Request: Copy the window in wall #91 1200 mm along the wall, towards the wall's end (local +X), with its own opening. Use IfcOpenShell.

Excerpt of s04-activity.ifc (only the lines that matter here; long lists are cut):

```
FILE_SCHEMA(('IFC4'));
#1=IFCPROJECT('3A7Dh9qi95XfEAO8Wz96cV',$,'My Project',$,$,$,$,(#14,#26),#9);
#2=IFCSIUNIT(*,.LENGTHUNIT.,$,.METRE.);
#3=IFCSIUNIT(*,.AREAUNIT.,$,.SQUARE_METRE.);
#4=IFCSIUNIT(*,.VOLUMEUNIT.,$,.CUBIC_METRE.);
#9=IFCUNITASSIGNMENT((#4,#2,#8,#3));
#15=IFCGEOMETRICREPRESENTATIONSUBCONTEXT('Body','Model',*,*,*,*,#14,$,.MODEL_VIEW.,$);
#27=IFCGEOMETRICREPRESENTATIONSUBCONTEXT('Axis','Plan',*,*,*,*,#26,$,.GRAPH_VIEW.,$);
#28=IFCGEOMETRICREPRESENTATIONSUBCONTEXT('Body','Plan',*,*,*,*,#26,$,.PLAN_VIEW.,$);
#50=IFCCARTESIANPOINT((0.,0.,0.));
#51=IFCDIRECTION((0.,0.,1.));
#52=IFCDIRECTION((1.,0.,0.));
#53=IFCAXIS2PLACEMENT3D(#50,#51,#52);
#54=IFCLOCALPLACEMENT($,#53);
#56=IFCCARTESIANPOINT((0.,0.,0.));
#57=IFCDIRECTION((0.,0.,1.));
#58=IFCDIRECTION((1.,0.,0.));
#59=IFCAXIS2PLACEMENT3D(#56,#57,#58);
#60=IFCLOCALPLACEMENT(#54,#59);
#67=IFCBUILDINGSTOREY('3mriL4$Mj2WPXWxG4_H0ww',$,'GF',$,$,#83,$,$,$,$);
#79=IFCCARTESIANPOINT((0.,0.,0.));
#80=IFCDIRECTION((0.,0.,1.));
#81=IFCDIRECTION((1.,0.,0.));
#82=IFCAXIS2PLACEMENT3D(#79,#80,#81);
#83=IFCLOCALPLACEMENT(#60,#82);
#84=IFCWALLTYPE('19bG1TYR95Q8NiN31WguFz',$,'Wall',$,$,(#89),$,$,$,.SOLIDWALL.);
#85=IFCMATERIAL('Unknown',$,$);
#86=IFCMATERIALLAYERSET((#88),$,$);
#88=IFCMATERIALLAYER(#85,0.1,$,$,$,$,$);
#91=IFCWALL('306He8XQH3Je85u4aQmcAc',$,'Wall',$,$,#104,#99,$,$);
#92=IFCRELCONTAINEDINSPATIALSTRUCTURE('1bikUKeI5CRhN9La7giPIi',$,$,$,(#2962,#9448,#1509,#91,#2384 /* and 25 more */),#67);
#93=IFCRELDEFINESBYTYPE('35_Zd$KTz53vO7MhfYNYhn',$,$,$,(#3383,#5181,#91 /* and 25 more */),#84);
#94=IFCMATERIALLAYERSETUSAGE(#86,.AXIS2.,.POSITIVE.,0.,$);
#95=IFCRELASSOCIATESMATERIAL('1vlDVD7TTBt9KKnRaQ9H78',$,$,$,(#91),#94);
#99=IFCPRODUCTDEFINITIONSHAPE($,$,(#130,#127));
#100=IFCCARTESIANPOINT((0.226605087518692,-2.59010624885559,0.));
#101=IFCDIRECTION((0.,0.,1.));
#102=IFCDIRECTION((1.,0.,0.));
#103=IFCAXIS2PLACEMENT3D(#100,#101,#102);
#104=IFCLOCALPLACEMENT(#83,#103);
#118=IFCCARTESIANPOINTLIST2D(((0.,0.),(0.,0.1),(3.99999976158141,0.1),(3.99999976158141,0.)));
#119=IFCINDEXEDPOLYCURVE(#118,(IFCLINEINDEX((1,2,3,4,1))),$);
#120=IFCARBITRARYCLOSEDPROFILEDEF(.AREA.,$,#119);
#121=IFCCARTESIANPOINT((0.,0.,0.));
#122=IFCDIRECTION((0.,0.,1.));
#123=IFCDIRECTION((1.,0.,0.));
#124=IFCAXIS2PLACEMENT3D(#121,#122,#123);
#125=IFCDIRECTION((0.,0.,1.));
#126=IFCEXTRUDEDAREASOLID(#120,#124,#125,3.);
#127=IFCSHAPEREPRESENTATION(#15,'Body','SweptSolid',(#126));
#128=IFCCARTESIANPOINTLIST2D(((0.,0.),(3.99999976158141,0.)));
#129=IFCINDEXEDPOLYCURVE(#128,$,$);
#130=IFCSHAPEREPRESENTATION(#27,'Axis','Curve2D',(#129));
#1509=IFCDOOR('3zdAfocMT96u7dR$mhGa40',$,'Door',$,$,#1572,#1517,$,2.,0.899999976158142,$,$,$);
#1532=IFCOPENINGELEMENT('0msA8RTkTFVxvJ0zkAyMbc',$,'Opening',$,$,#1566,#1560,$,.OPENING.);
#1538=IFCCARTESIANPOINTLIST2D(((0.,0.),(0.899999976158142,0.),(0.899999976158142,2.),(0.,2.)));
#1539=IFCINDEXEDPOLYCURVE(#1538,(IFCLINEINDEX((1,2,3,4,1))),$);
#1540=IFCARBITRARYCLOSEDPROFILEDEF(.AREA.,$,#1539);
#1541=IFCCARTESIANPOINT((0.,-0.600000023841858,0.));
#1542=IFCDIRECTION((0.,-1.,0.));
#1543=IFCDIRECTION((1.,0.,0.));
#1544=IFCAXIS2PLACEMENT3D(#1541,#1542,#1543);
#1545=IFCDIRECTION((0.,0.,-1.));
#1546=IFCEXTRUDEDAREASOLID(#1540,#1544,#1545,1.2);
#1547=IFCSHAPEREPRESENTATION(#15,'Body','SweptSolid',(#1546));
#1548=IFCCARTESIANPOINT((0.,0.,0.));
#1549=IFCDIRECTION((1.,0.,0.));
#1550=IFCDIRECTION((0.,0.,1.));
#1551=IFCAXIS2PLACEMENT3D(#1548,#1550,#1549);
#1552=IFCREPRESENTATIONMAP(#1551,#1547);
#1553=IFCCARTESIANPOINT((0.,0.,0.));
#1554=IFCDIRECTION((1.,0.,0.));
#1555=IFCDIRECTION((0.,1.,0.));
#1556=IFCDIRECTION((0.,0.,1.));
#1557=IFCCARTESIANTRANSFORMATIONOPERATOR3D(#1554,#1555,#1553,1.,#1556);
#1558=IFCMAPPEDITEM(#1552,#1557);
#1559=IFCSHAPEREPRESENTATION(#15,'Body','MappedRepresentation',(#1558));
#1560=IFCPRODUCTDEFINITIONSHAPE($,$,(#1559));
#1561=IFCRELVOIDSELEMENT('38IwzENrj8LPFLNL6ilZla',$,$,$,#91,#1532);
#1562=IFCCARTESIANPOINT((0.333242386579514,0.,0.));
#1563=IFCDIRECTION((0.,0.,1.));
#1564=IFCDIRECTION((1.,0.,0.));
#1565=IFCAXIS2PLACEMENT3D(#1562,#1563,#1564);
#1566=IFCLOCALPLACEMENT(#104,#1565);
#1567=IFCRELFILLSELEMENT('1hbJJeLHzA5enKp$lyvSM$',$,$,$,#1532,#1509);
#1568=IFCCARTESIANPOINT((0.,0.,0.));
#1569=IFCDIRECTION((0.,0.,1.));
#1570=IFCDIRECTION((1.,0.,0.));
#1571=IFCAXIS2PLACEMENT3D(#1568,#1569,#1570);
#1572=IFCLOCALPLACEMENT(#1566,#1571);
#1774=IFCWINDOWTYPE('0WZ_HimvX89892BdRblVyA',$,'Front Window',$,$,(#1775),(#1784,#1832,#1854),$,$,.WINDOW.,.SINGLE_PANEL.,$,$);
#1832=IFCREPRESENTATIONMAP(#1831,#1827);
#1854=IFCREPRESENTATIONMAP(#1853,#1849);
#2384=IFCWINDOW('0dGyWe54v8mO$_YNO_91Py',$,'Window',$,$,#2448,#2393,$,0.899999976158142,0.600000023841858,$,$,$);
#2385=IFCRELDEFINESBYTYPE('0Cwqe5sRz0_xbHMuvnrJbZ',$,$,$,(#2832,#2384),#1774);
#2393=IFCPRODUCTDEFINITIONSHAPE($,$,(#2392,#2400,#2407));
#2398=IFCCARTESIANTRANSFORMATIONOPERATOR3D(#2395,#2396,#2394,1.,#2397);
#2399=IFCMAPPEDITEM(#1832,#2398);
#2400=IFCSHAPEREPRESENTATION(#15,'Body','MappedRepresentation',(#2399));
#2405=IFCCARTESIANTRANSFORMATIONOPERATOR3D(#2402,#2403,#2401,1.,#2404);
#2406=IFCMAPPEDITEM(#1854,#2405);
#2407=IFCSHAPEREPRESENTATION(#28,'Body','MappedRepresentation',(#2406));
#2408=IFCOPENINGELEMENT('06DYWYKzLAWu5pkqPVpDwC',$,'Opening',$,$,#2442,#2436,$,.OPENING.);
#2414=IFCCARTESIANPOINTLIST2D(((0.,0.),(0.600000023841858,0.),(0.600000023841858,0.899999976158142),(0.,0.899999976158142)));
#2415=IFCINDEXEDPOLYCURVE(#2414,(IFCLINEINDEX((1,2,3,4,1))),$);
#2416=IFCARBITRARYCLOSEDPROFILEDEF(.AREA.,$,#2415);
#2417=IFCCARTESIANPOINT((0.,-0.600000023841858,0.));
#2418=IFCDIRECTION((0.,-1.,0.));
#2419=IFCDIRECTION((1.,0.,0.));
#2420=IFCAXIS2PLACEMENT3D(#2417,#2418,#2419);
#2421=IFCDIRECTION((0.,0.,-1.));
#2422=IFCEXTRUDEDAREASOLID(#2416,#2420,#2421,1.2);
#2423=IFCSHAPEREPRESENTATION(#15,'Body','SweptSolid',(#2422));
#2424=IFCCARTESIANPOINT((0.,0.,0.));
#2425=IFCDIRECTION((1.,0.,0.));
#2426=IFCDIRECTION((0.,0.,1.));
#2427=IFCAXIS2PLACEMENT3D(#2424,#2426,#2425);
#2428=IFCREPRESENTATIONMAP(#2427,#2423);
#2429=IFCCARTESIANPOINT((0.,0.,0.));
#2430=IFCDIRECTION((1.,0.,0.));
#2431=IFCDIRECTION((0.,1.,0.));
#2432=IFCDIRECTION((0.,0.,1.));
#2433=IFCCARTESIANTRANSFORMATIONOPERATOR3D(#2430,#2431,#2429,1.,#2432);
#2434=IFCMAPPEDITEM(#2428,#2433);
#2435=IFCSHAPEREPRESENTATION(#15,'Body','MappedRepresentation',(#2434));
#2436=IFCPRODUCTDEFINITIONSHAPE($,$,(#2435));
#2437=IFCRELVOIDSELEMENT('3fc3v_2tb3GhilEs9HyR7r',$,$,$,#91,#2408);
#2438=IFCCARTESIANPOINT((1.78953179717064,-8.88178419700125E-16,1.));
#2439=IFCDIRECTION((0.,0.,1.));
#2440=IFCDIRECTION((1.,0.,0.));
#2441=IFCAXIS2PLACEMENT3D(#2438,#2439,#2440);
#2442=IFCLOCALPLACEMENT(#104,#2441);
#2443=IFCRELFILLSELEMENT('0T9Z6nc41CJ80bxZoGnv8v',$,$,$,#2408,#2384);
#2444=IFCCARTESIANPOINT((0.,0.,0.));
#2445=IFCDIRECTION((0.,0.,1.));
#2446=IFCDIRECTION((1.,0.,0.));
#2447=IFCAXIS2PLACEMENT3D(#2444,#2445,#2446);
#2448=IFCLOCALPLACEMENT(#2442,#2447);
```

```python
import ifcopenshell
import ifcopenshell.api.feature
import ifcopenshell.api.geometry
import ifcopenshell.api.root
import ifcopenshell.geom
import ifcopenshell.util.element
import ifcopenshell.util.placement
import ifcopenshell.util.shape
import ifcopenshell.util.unit

model = ifcopenshell.open("s04-activity.ifc")
unit_scale = ifcopenshell.util.unit.calculate_unit_scale(model)
settings = ifcopenshell.geom.settings()


def volume(element):
    """Net volume in cubic metres, openings subtracted."""
    shape = ifcopenshell.geom.create_shape(settings, element)
    return ifcopenshell.util.shape.get_volume(shape.geometry)


window = model.by_guid("0dGyWe54v8mO$_YNO_91Py")
opening = window.FillsVoids[0].RelatingOpeningElement
wall = opening.VoidsElements[0].RelatingBuildingElement
before = volume(wall)
shift = ifcopenshell.util.placement.get_local_placement(wall.ObjectPlacement)[:3, 0] * 1.2 / unit_scale

# copy_class copies the void relationship, type, container and properties, but no geometry.
new_opening = ifcopenshell.api.root.copy_class(model, product=opening)
new_opening.Representation = ifcopenshell.util.element.copy_deep(
    model, opening.Representation, exclude=["IfcGeometricRepresentationContext", "IfcRepresentationMap"]
)
new_window = ifcopenshell.api.root.copy_class(model, product=window)
new_window.Representation = ifcopenshell.util.element.copy_deep(
    model, window.Representation, exclude=["IfcGeometricRepresentationContext", "IfcRepresentationMap"]
)
ifcopenshell.api.feature.add_filling(model, opening=new_opening, element=new_window)

for old, new in ((opening, new_opening), (window, new_window)):
    matrix = ifcopenshell.util.placement.get_local_placement(old.ObjectPlacement)
    matrix[:3, 3] += shift
    ifcopenshell.api.geometry.edit_object_placement(model, product=new, matrix=matrix, is_si=False)

after = volume(wall)

print(f"wall volume {before:.3f} -> {after:.3f} m3")

model.write("s04-activity_rev.ifc")
```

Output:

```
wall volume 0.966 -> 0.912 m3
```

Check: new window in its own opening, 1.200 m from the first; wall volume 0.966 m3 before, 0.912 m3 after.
